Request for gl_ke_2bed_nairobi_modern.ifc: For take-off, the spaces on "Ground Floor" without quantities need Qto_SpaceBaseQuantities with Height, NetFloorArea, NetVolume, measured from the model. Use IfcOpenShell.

First a look at what the model holds.

```python
import ifcopenshell
import ifcopenshell.util.element
import ifcopenshell.util.unit

model = ifcopenshell.open("gl_ke_2bed_nairobi_modern.ifc")
print(model.schema)
for unit_type in ("LENGTHUNIT", "AREAUNIT", "VOLUMEUNIT"):
    print(unit_type, ifcopenshell.util.unit.calculate_unit_scale(model, unit_type))
storey = next(s for s in model.by_type("IfcBuildingStorey") if s.Name == "Ground Floor")
spaces = [e for e in ifcopenshell.util.element.get_decomposition(storey) if e.is_a("IfcSpace")]
for e in sorted(spaces, key=lambda e: e.id()):
    print(e.id(), e.is_a(), e.Name, list(ifcopenshell.util.element.get_psets(e, qtos_only=True)), sep=" | ")
```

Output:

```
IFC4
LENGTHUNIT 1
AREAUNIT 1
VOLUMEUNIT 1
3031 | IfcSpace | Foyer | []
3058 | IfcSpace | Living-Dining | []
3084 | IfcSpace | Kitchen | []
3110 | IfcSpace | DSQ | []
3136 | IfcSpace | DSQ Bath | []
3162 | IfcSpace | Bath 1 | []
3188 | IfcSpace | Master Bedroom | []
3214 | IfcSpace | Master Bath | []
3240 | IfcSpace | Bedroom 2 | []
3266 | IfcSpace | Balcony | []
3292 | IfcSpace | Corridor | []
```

```python
import ifcopenshell
import ifcopenshell.api.pset
import ifcopenshell.geom
import ifcopenshell.util.element
import ifcopenshell.util.shape
import ifcopenshell.util.unit

model = ifcopenshell.open("gl_ke_2bed_nairobi_modern.ifc")
unit_scale = ifcopenshell.util.unit.calculate_unit_scale(model)
area_scale = ifcopenshell.util.unit.calculate_unit_scale(model, "AREAUNIT")
volume_scale = ifcopenshell.util.unit.calculate_unit_scale(model, "VOLUMEUNIT")
settings = ifcopenshell.geom.settings()

storey = next(s for s in model.by_type("IfcBuildingStorey") if s.Name == "Ground Floor")
spaces = [e for e in ifcopenshell.util.element.get_decomposition(storey) if e.is_a("IfcSpace")]

for e in sorted(spaces, key=lambda e: e.id()):
    if ifcopenshell.util.element.get_psets(e, qtos_only=True, should_inherit=False):
        continue
    # Geometry comes back in metres, in the element's own axes.
    shape = ifcopenshell.geom.create_shape(settings, e)
    values = {
        "Height": ifcopenshell.util.shape.get_z(shape.geometry) / unit_scale,
        "NetFloorArea": ifcopenshell.util.shape.get_footprint_area(shape.geometry) / area_scale,
        "NetVolume": ifcopenshell.util.shape.get_volume(shape.geometry) / volume_scale,
    }
    qto = ifcopenshell.api.pset.add_qto(model, product=e, name="Qto_SpaceBaseQuantities")
    ifcopenshell.api.pset.edit_qto(model, qto=qto, properties=values)
    print(e.id(), {k: round(v, 3) for k, v in values.items()})

model.write("gl_ke_2bed_nairobi_modern_v2.ifc")
```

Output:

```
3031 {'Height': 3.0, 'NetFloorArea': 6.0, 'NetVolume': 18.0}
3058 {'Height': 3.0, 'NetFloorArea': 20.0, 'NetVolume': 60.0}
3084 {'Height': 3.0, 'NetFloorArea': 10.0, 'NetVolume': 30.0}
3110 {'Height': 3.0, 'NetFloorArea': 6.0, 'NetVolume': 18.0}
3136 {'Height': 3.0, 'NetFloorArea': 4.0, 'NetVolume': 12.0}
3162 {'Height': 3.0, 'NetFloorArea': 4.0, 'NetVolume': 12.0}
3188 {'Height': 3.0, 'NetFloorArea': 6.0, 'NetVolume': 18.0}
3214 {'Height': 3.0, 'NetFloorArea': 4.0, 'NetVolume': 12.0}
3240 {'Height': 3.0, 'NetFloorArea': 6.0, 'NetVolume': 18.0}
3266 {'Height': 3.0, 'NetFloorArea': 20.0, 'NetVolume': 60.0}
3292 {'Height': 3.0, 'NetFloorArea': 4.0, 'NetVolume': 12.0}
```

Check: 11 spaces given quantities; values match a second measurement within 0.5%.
